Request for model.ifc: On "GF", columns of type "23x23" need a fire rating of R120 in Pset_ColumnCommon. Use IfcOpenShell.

First a look at what the model holds.

```python
import ifcopenshell
import ifcopenshell.util.element

model = ifcopenshell.open("model.ifc")
print(model.schema)
storey = next(s for s in model.by_type("IfcBuildingStorey") if s.Name == "GF")
columns = [e for e in ifcopenshell.util.element.get_decomposition(storey) if e.is_a("IfcColumn")]
seen = {}
for e in columns:
    element_type = ifcopenshell.util.element.get_type(e)
    key = (element_type.Name if element_type != e and element_type else None, ifcopenshell.util.element.get_pset(e, "Pset_ColumnCommon", "FireRating"))
    seen[key] = seen.get(key, 0) + 1
for (name, value), count in sorted(seen.items(), key=str):
    print(count, "x", name, "|", value)
```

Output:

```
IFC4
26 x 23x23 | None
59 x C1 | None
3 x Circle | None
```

```python
import ifcopenshell
import ifcopenshell.api.pset
import ifcopenshell.util.element

model = ifcopenshell.open("model.ifc")

storey = next(s for s in model.by_type("IfcBuildingStorey") if s.Name == "GF")
columns = [e for e in ifcopenshell.util.element.get_decomposition(storey) if e.is_a("IfcColumn")]

count = 0
for e in columns:
    element_type = ifcopenshell.util.element.get_type(e)
    if element_type in (None, e) or element_type.Name != "23x23":
        continue
    # add_pset returns the element's existing set when there is one.
    pset = ifcopenshell.api.pset.add_pset(model, product=e, name="Pset_ColumnCommon")
    ifcopenshell.api.pset.edit_pset(model, pset=pset, properties={"FireRating": "R120"})
    count += 1

print(count, "columns updated")

model.write("model_v2.ifc")
```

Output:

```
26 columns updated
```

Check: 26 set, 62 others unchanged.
